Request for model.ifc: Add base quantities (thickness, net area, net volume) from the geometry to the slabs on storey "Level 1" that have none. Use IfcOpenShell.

First a look at what the model holds.

```python
import ifcopenshell
import ifcopenshell.util.element
import ifcopenshell.util.unit

model = ifcopenshell.open("model.ifc")
print(model.schema)
for unit_type in ("LENGTHUNIT", "AREAUNIT", "VOLUMEUNIT"):
    print(unit_type, ifcopenshell.util.unit.calculate_unit_scale(model, unit_type))
storey = next(s for s in model.by_type("IfcBuildingStorey") if s.Name == "Level 1")
slabs = [e for e in ifcopenshell.util.element.get_decomposition(storey) if e.is_a("IfcSlab")]
for e in sorted(slabs, key=lambda e: e.id()):
    print(e.id(), e.is_a(), e.Name, list(ifcopenshell.util.element.get_psets(e, qtos_only=True)), sep=" | ")
```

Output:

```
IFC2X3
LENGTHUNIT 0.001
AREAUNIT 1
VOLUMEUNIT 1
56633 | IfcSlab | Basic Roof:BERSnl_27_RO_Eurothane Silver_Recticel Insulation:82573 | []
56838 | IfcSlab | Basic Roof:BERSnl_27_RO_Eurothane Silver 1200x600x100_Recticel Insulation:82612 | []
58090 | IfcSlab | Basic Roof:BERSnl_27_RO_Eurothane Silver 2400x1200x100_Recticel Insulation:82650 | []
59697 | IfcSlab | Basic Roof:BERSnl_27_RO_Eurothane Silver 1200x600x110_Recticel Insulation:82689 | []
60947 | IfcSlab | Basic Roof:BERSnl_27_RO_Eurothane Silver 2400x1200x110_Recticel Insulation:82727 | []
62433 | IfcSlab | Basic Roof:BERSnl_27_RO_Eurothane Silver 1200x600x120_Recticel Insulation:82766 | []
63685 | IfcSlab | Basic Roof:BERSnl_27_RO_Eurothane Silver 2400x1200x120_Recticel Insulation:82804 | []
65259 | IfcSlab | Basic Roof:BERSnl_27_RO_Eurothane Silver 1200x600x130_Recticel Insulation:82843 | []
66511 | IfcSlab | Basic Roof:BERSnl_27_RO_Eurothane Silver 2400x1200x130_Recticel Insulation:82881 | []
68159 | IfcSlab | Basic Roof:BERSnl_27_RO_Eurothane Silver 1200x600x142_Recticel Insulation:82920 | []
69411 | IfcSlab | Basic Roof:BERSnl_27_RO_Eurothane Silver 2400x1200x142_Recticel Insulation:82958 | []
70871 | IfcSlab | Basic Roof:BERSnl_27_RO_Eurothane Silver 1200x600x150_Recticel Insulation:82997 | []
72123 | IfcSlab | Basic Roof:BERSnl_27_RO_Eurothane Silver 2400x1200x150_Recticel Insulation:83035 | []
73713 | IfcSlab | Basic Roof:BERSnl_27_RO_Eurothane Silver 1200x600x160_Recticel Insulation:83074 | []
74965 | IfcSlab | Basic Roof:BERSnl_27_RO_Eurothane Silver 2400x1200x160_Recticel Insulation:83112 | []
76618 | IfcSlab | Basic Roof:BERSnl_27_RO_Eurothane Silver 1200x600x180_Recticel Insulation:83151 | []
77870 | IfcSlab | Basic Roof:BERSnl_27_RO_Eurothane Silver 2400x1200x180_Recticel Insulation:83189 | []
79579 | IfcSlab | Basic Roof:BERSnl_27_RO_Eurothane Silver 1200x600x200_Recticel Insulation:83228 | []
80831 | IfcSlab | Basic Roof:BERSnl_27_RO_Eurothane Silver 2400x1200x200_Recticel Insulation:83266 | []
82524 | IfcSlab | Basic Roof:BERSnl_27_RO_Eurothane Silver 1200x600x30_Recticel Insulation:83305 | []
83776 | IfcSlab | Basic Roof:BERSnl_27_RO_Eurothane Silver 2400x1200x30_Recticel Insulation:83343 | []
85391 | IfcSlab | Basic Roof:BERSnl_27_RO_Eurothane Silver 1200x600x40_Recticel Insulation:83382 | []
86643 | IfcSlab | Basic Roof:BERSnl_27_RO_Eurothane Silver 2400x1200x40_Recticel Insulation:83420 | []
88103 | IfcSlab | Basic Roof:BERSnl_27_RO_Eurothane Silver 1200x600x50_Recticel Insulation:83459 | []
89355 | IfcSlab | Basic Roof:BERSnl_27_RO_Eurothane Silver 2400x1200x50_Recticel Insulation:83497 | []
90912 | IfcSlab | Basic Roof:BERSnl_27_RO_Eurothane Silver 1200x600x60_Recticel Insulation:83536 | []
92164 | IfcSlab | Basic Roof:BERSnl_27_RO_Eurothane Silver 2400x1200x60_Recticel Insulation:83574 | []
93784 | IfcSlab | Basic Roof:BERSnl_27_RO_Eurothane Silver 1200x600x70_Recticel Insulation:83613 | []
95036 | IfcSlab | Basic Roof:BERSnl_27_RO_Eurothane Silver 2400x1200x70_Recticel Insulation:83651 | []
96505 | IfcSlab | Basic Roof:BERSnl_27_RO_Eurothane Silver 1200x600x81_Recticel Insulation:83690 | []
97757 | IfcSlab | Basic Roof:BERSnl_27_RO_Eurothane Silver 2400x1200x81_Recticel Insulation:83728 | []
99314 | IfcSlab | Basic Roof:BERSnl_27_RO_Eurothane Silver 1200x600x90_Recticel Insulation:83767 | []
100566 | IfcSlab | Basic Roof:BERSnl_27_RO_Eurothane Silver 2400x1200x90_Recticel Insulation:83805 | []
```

```python
import ifcopenshell
import ifcopenshell.api.pset
import ifcopenshell.geom
import ifcopenshell.util.element
import ifcopenshell.util.shape
import ifcopenshell.util.unit

model = ifcopenshell.open("model.ifc")
unit_scale = ifcopenshell.util.unit.calculate_unit_scale(model)
area_scale = ifcopenshell.util.unit.calculate_unit_scale(model, "AREAUNIT")
volume_scale = ifcopenshell.util.unit.calculate_unit_scale(model, "VOLUMEUNIT")
settings = ifcopenshell.geom.settings()

storey = next(s for s in model.by_type("IfcBuildingStorey") if s.Name == "Level 1")
slabs = [e for e in ifcopenshell.util.element.get_decomposition(storey) if e.is_a("IfcSlab")]

for e in sorted(slabs, key=lambda e: e.id()):
    if ifcopenshell.util.element.get_psets(e, qtos_only=True, should_inherit=False):
        continue
    # Geometry comes back in metres, in the element's own axes.
    shape = ifcopenshell.geom.create_shape(settings, e)
    values = {
        "Width": ifcopenshell.util.shape.get_z(shape.geometry) / unit_scale,
        "NetArea": ifcopenshell.util.shape.get_footprint_area(shape.geometry) / area_scale,
        "NetVolume": ifcopenshell.util.shape.get_volume(shape.geometry) / volume_scale,
    }
    qto = ifcopenshell.api.pset.add_qto(model, product=e, name="BaseQuantities")
    ifcopenshell.api.pset.edit_qto(model, qto=qto, properties=values)
    print(e.id(), {k: round(v, 3) for k, v in values.items()})

model.write("model_edited.ifc")
```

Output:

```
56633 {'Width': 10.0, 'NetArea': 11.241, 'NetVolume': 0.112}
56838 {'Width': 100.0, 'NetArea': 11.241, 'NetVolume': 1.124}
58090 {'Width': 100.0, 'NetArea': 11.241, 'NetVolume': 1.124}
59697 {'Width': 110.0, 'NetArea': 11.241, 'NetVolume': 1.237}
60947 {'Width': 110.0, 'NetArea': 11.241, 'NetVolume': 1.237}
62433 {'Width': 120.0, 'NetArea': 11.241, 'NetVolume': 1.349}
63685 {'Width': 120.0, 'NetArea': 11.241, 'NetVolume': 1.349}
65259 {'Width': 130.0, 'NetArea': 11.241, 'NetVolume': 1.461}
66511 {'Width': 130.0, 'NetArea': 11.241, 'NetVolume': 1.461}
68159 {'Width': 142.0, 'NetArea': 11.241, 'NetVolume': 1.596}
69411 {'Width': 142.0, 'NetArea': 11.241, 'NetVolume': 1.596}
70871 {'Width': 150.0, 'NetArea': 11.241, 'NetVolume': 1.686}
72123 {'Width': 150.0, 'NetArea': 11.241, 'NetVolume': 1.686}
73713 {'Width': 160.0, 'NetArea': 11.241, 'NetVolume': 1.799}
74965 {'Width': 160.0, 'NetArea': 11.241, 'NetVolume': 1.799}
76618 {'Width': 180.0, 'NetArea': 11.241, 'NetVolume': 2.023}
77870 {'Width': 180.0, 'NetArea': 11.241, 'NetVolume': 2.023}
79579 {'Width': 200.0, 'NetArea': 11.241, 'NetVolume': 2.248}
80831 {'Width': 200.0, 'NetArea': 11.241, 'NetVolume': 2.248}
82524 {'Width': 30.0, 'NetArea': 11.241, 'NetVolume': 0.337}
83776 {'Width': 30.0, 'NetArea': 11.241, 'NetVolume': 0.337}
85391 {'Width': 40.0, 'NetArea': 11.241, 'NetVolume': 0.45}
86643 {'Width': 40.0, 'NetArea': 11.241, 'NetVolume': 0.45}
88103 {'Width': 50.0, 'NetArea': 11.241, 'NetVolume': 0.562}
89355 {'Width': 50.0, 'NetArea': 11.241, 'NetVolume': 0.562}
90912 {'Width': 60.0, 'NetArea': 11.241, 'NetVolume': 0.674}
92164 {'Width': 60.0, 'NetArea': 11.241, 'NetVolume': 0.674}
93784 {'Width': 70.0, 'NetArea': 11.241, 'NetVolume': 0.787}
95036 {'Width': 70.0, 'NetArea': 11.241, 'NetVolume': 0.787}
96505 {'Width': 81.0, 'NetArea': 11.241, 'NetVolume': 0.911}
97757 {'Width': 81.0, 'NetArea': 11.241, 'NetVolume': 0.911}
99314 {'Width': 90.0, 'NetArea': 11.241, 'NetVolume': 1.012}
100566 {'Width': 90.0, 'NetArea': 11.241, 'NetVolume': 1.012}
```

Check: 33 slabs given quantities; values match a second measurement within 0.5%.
